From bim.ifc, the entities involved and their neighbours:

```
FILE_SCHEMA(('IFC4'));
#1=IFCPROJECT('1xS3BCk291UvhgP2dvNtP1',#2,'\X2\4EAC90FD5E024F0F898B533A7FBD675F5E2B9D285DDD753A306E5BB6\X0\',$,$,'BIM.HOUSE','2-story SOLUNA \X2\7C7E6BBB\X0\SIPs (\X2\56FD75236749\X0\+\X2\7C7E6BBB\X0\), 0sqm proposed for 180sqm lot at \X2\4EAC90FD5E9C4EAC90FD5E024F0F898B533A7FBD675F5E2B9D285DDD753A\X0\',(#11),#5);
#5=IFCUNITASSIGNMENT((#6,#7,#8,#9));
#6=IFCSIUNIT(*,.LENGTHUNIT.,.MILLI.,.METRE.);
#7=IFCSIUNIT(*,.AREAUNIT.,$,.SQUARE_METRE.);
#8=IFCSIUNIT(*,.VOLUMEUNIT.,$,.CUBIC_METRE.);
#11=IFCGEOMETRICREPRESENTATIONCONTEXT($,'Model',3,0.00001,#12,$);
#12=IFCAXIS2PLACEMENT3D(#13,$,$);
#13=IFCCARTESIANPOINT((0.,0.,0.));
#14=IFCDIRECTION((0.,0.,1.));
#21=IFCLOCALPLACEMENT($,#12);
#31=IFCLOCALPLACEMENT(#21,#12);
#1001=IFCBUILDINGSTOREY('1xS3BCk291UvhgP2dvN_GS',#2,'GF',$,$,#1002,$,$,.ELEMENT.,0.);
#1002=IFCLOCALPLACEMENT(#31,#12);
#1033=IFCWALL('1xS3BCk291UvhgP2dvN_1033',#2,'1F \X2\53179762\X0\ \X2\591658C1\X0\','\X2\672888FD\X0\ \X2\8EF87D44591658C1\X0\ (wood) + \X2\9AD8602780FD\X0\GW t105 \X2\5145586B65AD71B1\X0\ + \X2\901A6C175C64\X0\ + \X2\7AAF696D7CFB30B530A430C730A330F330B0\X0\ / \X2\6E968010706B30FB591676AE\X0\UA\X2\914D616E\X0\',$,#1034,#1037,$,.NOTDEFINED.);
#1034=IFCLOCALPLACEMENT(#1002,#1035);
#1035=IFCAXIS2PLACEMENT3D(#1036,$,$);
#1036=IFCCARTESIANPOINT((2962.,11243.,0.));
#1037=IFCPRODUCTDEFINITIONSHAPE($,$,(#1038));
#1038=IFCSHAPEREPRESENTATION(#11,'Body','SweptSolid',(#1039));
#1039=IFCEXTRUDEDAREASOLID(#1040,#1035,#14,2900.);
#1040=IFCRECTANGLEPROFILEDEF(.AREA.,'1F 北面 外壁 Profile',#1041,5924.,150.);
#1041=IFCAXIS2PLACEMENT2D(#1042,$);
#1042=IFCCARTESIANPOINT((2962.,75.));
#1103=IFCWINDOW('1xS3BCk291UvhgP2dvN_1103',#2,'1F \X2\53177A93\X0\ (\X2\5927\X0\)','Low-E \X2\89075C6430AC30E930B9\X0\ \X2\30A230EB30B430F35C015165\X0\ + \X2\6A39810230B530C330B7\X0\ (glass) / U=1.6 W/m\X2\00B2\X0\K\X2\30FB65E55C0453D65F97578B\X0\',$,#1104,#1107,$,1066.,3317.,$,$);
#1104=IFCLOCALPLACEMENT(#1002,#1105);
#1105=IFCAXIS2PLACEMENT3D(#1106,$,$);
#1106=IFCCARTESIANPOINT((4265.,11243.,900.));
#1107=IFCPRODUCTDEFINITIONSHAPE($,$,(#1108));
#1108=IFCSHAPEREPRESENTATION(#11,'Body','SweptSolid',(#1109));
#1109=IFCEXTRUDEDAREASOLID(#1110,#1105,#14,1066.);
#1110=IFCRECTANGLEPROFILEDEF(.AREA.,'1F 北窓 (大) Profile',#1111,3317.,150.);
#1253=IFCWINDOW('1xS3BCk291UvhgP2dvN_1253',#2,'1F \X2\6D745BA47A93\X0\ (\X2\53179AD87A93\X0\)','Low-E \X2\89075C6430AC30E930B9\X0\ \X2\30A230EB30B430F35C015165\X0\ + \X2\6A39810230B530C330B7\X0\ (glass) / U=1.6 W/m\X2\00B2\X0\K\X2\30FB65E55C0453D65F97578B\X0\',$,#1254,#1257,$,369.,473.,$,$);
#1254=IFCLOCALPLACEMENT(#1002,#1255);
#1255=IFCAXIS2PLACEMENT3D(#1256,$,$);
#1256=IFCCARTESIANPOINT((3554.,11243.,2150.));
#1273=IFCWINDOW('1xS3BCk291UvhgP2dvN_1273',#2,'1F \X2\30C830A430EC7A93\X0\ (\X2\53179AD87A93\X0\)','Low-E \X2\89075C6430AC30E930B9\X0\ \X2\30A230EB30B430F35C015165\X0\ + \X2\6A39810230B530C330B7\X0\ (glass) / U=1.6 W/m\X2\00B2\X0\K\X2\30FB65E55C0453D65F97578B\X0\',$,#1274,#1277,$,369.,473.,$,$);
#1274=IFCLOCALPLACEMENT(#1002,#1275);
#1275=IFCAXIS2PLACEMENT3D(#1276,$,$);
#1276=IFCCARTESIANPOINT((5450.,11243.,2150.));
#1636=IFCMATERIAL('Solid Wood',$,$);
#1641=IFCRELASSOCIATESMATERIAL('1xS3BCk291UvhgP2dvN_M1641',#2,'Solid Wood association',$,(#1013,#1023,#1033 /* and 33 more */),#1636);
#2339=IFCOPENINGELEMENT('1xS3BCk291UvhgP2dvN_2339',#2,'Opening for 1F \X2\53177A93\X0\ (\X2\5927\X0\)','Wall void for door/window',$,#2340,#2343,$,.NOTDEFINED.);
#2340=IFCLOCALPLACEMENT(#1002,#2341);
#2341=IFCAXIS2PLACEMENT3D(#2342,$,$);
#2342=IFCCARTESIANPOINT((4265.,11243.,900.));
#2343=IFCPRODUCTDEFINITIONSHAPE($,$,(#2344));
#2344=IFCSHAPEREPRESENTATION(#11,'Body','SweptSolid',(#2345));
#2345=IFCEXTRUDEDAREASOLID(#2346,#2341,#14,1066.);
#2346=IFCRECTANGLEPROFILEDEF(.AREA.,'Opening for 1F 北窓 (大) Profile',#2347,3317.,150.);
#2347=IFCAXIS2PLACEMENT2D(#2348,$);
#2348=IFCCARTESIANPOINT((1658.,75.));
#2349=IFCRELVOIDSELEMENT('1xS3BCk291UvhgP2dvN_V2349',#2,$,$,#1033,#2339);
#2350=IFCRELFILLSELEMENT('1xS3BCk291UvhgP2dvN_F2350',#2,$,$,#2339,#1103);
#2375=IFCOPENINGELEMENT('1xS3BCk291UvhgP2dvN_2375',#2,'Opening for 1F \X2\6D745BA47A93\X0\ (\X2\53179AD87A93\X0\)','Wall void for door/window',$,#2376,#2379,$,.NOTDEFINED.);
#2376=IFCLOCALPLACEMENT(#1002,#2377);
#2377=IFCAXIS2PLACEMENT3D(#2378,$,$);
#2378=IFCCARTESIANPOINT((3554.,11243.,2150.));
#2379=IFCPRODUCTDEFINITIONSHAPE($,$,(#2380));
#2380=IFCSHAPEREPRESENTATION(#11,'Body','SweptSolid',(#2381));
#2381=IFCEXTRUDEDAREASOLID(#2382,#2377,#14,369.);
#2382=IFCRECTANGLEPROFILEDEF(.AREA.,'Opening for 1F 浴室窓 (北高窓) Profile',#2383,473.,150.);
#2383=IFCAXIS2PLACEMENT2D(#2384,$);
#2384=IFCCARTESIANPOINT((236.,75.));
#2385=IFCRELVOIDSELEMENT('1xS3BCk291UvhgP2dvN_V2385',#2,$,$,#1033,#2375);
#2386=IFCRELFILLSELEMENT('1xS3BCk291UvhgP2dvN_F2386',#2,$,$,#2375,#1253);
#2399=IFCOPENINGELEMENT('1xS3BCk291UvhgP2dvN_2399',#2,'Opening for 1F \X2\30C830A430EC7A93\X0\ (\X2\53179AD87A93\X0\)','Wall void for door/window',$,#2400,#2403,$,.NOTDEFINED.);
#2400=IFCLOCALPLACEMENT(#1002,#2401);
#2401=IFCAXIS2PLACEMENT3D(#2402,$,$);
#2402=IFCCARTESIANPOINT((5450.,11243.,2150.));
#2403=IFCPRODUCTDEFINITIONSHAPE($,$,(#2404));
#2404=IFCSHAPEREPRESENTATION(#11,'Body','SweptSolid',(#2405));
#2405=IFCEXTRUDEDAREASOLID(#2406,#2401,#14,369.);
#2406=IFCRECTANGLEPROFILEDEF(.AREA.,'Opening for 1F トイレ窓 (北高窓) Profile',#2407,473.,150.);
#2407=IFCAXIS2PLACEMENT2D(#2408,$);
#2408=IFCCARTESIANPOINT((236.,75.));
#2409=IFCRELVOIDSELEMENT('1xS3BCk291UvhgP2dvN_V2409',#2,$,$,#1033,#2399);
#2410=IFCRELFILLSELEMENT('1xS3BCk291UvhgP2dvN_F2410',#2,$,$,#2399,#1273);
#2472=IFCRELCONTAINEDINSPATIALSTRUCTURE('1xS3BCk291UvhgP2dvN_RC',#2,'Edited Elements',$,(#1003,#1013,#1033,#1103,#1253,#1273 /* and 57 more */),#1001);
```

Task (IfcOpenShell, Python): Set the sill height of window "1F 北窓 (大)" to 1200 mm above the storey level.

```python
import numpy as np
import ifcopenshell
import ifcopenshell.api.geometry
import ifcopenshell.geom
import ifcopenshell.util.element
import ifcopenshell.util.placement
import ifcopenshell.util.shape
import ifcopenshell.util.unit

model = ifcopenshell.open("bim.ifc")
unit_scale = ifcopenshell.util.unit.calculate_unit_scale(model)

window = model.by_guid("1xS3BCk291UvhgP2dvN_1103")
opening = window.FillsVoids[0].RelatingOpeningElement
storey = ifcopenshell.util.element.get_container(window, ifc_class="IfcBuildingStorey")
level = ifcopenshell.util.placement.get_local_placement(storey.ObjectPlacement)[2, 3]

# The opening's origin need not be at the sill, so measure its lowest point.
shape = ifcopenshell.geom.create_shape(ifcopenshell.geom.settings(), opening)
bottom = ifcopenshell.util.shape.get_shape_bottom_elevation(shape, shape.geometry) / unit_scale
dz = level + 1200.0 - bottom

shift = np.array([0.0, 0.0, dz])
# The window is not placed relative to its opening, so move both.
for product in (opening, window):
    matrix = ifcopenshell.util.placement.get_local_placement(product.ObjectPlacement)
    matrix[:3, 3] += shift
    ifcopenshell.api.geometry.edit_object_placement(model, product=product, matrix=matrix, is_si=False)

print(f"moved by {dz * unit_scale:+.3f} m")

model.write("bim-out.ifc")
```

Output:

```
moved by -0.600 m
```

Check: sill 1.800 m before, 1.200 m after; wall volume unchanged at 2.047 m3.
